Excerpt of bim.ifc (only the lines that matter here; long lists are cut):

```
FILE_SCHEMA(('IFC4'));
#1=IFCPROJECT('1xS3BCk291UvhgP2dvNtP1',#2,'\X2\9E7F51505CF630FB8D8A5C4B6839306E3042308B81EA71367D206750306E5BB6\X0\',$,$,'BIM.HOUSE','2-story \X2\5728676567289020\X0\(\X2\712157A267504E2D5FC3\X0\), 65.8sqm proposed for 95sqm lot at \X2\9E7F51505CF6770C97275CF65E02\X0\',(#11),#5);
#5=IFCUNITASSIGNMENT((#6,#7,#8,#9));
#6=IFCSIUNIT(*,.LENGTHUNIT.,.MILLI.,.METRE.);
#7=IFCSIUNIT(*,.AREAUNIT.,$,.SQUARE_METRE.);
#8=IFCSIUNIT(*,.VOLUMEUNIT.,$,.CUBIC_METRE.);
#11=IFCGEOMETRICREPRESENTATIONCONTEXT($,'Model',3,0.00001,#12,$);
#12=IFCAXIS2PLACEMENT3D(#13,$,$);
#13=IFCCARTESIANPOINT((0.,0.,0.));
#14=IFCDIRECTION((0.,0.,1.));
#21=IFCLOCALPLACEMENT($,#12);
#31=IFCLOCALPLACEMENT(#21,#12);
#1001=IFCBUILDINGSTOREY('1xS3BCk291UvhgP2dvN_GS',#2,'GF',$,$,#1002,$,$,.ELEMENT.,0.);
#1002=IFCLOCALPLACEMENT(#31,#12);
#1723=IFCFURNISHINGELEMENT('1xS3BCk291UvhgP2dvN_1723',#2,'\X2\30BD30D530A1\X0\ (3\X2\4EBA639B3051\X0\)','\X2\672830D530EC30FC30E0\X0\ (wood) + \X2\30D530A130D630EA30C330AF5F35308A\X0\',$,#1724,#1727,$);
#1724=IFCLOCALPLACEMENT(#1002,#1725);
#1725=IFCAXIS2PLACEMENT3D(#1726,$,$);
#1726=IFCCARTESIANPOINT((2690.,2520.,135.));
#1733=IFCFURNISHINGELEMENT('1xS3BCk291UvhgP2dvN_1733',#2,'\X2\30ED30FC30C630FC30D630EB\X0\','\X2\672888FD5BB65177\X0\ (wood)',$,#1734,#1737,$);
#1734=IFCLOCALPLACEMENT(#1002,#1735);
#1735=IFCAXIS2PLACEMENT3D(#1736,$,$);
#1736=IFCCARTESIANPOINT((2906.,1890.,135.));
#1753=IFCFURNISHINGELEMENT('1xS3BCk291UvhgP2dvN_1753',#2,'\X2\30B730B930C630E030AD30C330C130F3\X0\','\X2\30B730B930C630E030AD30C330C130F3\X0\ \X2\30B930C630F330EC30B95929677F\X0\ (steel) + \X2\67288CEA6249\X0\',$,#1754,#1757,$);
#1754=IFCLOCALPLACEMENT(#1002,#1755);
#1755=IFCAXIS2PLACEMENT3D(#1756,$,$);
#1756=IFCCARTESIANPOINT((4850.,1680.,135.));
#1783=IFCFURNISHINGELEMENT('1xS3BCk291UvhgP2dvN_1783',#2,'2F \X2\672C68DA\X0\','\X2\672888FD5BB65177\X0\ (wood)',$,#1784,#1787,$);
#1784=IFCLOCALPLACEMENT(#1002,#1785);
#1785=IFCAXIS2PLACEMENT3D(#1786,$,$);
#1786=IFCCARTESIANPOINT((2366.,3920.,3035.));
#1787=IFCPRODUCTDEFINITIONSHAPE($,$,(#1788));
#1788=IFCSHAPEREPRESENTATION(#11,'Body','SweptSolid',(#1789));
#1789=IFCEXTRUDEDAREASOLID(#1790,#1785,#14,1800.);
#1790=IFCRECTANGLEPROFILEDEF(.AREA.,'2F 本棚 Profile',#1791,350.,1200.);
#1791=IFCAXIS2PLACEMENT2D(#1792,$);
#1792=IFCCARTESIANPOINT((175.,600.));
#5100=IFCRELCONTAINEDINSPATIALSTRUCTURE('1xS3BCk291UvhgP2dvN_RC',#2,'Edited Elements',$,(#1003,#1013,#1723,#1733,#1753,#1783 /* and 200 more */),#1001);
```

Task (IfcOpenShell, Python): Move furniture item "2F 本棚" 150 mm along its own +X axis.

```python
import ifcopenshell
import ifcopenshell.api.geometry
import ifcopenshell.util.placement
import ifcopenshell.util.unit

model = ifcopenshell.open("bim.ifc")
unit_scale = ifcopenshell.util.unit.calculate_unit_scale(model)

item = model.by_guid("1xS3BCk291UvhgP2dvN_1783")
matrix = ifcopenshell.util.placement.get_local_placement(item.ObjectPlacement)
matrix[:3, 3] += matrix[:3, 0] * 0.15 / unit_scale
ifcopenshell.api.geometry.edit_object_placement(model, product=item, matrix=matrix, is_si=False)

print(ifcopenshell.util.placement.get_local_placement(item.ObjectPlacement).round(3) + 0.0)

model.write("bim_updated.ifc")
```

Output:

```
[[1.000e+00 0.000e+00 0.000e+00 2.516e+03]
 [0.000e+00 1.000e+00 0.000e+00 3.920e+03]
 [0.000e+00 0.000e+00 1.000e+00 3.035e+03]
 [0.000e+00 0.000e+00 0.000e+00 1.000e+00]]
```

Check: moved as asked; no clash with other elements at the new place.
